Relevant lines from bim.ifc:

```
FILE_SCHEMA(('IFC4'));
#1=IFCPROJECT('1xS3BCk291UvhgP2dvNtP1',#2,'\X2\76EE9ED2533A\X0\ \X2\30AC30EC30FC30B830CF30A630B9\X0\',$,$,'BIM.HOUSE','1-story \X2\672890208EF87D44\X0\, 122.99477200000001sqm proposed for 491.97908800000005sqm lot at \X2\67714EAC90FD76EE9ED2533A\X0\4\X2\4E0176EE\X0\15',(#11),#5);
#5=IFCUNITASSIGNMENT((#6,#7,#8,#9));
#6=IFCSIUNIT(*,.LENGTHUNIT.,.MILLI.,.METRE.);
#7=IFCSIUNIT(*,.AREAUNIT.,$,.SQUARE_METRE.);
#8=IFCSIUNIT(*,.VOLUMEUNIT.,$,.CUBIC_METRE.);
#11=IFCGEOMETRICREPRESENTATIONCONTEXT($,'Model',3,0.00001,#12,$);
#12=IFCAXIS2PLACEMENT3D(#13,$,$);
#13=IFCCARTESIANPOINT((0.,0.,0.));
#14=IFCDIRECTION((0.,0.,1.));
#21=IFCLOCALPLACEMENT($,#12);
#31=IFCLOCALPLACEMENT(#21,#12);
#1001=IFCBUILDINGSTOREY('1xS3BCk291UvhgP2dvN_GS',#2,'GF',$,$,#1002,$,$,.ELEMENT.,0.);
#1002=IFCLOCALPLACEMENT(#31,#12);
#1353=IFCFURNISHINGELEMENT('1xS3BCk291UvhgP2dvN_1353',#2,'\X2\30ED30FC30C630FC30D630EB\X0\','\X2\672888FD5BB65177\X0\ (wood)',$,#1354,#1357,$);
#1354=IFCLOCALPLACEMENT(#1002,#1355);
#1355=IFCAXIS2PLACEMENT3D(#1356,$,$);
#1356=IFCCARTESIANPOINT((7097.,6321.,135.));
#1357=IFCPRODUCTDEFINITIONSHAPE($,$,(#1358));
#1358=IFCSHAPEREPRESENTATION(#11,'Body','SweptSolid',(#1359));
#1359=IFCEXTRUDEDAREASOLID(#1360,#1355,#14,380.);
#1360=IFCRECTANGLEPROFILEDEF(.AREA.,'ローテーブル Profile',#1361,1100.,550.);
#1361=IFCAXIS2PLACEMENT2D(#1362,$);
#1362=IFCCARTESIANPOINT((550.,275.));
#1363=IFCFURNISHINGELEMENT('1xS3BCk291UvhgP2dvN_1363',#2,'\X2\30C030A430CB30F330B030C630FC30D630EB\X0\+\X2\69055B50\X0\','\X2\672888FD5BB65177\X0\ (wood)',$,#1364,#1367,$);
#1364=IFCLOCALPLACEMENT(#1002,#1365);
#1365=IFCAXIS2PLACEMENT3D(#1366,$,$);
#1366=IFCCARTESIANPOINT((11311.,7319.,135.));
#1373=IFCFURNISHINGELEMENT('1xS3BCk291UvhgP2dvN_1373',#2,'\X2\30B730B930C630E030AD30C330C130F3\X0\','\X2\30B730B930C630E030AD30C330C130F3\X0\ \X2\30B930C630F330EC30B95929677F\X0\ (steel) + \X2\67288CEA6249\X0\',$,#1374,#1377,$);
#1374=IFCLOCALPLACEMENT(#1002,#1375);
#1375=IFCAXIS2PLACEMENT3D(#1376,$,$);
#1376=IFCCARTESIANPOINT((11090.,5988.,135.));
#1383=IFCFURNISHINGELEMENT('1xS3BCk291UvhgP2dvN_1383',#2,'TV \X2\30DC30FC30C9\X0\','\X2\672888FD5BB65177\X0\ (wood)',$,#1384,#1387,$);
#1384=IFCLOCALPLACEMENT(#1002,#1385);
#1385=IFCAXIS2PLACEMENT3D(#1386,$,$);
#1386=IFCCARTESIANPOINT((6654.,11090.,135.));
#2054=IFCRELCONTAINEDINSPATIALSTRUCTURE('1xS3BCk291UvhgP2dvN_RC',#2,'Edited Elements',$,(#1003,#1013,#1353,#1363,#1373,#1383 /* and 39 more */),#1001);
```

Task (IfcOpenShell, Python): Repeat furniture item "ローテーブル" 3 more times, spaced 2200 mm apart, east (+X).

```python
import numpy as np
import ifcopenshell
import ifcopenshell.api.geometry
import ifcopenshell.api.root
import ifcopenshell.util.element
import ifcopenshell.util.placement

model = ifcopenshell.open("bim.ifc")


def reuse_history(source, copy):
    """copy_class also copies each property set's owner history, people and application; keep the originals."""
    for rel in copy.IsDefinedBy:
        if rel.is_a("IfcRelDefinesByProperties") and (history := rel.RelatingPropertyDefinition.OwnerHistory):
            rel.RelatingPropertyDefinition.OwnerHistory = source.OwnerHistory
            ifcopenshell.util.element.remove_deep2(model, history)


source = model.by_guid("1xS3BCk291UvhgP2dvN_1353")
base = ifcopenshell.util.placement.get_local_placement(source.ObjectPlacement)
step = np.array([1.0, 0.0, 0.0]) * 2200.0

for i in range(1, 4):
    copy = ifcopenshell.api.root.copy_class(model, product=source)
    copy.Representation = ifcopenshell.util.element.copy_deep(
        model, source.Representation, exclude=["IfcGeometricRepresentationContext", "IfcRepresentationMap"]
    )
    reuse_history(source, copy)
    matrix = base.copy()
    matrix[:3, 3] += i * step
    print("added at", matrix[:3, 3].round(3) + 0.0)
    ifcopenshell.api.geometry.edit_object_placement(model, product=copy, matrix=matrix, is_si=False)

model.write("bim_edited.ifc")
```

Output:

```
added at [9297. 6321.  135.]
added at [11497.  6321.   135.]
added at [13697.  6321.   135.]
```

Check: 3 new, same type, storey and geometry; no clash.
